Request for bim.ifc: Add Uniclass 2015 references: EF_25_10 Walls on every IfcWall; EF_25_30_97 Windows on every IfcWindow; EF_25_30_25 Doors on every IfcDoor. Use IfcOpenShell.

First a look at what the model holds.

```python
import ifcopenshell

model = ifcopenshell.open("bim.ifc")
print(model.schema)
print("classifications:", [c.Name for c in model.by_type("IfcClassification")])
for ifc_class in ("IfcDoor", "IfcRoof", "IfcStair", "IfcWall", "IfcWindow"):
    print(ifc_class, len(model.by_type(ifc_class)))
```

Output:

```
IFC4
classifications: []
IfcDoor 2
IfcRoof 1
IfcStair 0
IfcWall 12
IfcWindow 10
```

```python
import ifcopenshell
import ifcopenshell.api.classification

model = ifcopenshell.open("bim.ifc")

system = ifcopenshell.api.classification.add_classification(model, classification="Uniclass 2015")

codes = {
    "IfcWall": ("EF_25_10", "Walls"),
    "IfcWindow": ("EF_25_30_97", "Windows"),
    "IfcDoor": ("EF_25_30_25", "Doors"),
}
for ifc_class, (code, name) in codes.items():
    products = model.by_type(ifc_class)
    ifcopenshell.api.classification.add_reference(
        model, products=products, classification=system, identification=code, name=name
    )
    print(code, len(products))

model.write("bim_v2.ifc")
```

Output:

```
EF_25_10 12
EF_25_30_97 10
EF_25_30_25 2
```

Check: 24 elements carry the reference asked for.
